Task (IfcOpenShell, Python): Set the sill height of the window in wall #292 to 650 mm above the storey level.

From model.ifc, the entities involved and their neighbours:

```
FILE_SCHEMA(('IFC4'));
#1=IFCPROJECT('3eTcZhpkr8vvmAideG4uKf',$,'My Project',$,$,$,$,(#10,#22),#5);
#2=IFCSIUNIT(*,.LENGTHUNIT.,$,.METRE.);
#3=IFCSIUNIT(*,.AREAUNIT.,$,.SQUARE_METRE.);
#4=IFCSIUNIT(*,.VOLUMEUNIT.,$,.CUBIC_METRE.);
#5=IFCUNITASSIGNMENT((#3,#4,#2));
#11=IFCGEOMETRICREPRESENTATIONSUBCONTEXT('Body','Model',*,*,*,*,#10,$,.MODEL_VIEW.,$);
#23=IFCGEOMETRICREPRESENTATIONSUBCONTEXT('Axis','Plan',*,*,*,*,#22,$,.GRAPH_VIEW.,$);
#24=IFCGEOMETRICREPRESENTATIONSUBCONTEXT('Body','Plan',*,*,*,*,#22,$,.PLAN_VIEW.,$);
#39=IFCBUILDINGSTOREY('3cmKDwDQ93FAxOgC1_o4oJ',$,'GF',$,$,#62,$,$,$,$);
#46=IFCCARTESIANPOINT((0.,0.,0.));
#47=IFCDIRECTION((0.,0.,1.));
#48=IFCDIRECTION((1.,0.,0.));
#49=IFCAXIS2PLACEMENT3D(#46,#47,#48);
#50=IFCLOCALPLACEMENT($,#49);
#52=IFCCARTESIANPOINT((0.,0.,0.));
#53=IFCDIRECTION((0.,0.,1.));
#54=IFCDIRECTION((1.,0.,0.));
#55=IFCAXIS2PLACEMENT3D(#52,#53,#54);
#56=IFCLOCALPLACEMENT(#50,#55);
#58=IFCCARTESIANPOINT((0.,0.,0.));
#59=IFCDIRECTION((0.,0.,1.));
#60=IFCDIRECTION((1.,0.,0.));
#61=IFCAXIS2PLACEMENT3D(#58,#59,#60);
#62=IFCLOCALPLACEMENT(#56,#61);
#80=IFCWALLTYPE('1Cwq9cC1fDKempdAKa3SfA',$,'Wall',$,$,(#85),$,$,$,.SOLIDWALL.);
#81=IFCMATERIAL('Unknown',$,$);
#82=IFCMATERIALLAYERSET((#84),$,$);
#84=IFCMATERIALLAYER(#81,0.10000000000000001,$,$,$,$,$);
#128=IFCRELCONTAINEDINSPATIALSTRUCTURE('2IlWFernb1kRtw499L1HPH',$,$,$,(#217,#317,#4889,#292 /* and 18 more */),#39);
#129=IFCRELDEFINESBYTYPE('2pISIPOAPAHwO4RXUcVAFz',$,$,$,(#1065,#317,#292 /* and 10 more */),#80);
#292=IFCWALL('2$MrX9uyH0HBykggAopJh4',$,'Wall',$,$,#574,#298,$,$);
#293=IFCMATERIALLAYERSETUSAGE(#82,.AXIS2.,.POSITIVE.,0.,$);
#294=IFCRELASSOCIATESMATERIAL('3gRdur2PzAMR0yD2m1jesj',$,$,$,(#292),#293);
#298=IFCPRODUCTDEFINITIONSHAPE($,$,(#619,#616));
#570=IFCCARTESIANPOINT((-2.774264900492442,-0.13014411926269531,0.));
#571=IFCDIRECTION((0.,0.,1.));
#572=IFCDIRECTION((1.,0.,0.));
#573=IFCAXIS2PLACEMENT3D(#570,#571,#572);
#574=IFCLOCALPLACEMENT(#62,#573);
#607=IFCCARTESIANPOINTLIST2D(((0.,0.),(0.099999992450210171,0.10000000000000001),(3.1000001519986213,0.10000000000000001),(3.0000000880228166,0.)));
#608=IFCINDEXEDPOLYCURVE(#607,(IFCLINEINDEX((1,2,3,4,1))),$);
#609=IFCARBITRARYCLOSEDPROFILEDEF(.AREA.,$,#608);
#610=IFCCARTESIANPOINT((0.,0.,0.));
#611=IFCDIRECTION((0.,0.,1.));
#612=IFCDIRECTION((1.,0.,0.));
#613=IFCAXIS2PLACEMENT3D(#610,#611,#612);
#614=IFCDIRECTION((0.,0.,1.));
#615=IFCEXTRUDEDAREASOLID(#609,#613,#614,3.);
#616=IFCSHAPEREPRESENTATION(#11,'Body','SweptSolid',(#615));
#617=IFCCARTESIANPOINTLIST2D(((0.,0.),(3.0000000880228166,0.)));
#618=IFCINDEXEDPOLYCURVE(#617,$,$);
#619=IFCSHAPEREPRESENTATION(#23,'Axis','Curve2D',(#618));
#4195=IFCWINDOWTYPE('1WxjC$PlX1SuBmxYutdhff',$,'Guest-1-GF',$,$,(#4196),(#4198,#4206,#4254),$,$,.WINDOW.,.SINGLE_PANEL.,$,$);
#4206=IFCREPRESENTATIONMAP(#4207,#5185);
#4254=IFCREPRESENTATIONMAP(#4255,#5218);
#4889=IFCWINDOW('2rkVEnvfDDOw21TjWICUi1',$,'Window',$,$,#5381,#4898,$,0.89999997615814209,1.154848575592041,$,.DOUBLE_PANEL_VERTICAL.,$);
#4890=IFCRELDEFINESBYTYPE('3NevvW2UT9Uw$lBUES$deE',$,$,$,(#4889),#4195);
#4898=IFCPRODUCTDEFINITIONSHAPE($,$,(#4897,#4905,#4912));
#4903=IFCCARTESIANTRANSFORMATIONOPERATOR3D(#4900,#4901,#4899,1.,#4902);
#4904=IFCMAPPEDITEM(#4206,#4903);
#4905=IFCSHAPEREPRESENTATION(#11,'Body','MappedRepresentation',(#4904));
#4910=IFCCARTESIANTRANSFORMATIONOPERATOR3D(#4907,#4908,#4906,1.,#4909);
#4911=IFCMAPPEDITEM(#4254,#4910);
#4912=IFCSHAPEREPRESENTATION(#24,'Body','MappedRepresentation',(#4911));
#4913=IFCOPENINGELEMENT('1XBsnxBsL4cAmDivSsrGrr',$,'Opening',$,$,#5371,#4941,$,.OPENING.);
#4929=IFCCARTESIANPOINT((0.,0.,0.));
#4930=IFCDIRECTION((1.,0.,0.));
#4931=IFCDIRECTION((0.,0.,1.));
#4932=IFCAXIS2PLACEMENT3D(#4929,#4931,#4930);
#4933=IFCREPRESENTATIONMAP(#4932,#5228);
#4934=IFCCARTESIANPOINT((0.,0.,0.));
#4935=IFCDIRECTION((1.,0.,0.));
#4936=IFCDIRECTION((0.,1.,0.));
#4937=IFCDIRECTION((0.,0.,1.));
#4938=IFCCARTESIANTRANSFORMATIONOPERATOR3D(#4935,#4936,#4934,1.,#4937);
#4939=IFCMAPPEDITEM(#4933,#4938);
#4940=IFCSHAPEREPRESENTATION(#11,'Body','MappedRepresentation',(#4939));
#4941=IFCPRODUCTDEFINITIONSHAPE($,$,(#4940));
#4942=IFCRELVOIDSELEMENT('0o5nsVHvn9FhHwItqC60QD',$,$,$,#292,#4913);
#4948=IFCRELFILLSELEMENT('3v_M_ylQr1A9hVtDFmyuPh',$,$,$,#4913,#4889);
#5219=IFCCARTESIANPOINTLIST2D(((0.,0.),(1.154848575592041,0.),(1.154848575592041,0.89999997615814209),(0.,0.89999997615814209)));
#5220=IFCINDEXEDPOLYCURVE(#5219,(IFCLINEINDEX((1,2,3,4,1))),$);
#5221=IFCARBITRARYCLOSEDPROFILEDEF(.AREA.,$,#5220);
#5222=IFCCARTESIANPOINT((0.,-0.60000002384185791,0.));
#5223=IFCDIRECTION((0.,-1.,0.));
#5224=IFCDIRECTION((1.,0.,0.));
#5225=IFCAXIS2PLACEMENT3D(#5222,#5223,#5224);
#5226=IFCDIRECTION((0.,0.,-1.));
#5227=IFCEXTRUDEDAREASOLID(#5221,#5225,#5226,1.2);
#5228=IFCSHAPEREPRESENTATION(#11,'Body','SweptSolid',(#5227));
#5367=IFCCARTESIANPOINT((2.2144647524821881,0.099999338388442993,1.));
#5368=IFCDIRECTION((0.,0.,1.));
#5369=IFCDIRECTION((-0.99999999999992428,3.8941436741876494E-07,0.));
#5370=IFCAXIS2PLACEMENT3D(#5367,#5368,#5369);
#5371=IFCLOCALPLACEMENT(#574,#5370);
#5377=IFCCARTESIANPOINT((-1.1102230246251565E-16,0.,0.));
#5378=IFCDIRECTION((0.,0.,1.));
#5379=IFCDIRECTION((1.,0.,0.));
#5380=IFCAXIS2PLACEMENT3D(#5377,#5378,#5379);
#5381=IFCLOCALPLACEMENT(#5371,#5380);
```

```python
import numpy as np
import ifcopenshell
import ifcopenshell.api.geometry
import ifcopenshell.geom
import ifcopenshell.util.element
import ifcopenshell.util.placement
import ifcopenshell.util.shape
import ifcopenshell.util.unit

model = ifcopenshell.open("model.ifc")
unit_scale = ifcopenshell.util.unit.calculate_unit_scale(model)

window = model.by_guid("2rkVEnvfDDOw21TjWICUi1")
opening = window.FillsVoids[0].RelatingOpeningElement
storey = ifcopenshell.util.element.get_container(window, ifc_class="IfcBuildingStorey")
level = ifcopenshell.util.placement.get_local_placement(storey.ObjectPlacement)[2, 3]

# The opening's origin need not be at the sill, so measure its lowest point.
shape = ifcopenshell.geom.create_shape(ifcopenshell.geom.settings(), opening)
bottom = ifcopenshell.util.shape.get_shape_bottom_elevation(shape, shape.geometry) / unit_scale
dz = level + 0.65 / unit_scale - bottom

shift = np.array([0.0, 0.0, dz])
# The window is placed relative to its opening, so it follows when the opening moves.
matrix = ifcopenshell.util.placement.get_local_placement(opening.ObjectPlacement)
matrix[:3, 3] += shift
ifcopenshell.api.geometry.edit_object_placement(
    model, product=opening, matrix=matrix, is_si=False, should_transform_children=True
)

print(f"moved by {dz * unit_scale:+.3f} m")

model.write("model_v2.ifc")
```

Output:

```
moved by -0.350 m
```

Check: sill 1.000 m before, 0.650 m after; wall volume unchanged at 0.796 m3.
